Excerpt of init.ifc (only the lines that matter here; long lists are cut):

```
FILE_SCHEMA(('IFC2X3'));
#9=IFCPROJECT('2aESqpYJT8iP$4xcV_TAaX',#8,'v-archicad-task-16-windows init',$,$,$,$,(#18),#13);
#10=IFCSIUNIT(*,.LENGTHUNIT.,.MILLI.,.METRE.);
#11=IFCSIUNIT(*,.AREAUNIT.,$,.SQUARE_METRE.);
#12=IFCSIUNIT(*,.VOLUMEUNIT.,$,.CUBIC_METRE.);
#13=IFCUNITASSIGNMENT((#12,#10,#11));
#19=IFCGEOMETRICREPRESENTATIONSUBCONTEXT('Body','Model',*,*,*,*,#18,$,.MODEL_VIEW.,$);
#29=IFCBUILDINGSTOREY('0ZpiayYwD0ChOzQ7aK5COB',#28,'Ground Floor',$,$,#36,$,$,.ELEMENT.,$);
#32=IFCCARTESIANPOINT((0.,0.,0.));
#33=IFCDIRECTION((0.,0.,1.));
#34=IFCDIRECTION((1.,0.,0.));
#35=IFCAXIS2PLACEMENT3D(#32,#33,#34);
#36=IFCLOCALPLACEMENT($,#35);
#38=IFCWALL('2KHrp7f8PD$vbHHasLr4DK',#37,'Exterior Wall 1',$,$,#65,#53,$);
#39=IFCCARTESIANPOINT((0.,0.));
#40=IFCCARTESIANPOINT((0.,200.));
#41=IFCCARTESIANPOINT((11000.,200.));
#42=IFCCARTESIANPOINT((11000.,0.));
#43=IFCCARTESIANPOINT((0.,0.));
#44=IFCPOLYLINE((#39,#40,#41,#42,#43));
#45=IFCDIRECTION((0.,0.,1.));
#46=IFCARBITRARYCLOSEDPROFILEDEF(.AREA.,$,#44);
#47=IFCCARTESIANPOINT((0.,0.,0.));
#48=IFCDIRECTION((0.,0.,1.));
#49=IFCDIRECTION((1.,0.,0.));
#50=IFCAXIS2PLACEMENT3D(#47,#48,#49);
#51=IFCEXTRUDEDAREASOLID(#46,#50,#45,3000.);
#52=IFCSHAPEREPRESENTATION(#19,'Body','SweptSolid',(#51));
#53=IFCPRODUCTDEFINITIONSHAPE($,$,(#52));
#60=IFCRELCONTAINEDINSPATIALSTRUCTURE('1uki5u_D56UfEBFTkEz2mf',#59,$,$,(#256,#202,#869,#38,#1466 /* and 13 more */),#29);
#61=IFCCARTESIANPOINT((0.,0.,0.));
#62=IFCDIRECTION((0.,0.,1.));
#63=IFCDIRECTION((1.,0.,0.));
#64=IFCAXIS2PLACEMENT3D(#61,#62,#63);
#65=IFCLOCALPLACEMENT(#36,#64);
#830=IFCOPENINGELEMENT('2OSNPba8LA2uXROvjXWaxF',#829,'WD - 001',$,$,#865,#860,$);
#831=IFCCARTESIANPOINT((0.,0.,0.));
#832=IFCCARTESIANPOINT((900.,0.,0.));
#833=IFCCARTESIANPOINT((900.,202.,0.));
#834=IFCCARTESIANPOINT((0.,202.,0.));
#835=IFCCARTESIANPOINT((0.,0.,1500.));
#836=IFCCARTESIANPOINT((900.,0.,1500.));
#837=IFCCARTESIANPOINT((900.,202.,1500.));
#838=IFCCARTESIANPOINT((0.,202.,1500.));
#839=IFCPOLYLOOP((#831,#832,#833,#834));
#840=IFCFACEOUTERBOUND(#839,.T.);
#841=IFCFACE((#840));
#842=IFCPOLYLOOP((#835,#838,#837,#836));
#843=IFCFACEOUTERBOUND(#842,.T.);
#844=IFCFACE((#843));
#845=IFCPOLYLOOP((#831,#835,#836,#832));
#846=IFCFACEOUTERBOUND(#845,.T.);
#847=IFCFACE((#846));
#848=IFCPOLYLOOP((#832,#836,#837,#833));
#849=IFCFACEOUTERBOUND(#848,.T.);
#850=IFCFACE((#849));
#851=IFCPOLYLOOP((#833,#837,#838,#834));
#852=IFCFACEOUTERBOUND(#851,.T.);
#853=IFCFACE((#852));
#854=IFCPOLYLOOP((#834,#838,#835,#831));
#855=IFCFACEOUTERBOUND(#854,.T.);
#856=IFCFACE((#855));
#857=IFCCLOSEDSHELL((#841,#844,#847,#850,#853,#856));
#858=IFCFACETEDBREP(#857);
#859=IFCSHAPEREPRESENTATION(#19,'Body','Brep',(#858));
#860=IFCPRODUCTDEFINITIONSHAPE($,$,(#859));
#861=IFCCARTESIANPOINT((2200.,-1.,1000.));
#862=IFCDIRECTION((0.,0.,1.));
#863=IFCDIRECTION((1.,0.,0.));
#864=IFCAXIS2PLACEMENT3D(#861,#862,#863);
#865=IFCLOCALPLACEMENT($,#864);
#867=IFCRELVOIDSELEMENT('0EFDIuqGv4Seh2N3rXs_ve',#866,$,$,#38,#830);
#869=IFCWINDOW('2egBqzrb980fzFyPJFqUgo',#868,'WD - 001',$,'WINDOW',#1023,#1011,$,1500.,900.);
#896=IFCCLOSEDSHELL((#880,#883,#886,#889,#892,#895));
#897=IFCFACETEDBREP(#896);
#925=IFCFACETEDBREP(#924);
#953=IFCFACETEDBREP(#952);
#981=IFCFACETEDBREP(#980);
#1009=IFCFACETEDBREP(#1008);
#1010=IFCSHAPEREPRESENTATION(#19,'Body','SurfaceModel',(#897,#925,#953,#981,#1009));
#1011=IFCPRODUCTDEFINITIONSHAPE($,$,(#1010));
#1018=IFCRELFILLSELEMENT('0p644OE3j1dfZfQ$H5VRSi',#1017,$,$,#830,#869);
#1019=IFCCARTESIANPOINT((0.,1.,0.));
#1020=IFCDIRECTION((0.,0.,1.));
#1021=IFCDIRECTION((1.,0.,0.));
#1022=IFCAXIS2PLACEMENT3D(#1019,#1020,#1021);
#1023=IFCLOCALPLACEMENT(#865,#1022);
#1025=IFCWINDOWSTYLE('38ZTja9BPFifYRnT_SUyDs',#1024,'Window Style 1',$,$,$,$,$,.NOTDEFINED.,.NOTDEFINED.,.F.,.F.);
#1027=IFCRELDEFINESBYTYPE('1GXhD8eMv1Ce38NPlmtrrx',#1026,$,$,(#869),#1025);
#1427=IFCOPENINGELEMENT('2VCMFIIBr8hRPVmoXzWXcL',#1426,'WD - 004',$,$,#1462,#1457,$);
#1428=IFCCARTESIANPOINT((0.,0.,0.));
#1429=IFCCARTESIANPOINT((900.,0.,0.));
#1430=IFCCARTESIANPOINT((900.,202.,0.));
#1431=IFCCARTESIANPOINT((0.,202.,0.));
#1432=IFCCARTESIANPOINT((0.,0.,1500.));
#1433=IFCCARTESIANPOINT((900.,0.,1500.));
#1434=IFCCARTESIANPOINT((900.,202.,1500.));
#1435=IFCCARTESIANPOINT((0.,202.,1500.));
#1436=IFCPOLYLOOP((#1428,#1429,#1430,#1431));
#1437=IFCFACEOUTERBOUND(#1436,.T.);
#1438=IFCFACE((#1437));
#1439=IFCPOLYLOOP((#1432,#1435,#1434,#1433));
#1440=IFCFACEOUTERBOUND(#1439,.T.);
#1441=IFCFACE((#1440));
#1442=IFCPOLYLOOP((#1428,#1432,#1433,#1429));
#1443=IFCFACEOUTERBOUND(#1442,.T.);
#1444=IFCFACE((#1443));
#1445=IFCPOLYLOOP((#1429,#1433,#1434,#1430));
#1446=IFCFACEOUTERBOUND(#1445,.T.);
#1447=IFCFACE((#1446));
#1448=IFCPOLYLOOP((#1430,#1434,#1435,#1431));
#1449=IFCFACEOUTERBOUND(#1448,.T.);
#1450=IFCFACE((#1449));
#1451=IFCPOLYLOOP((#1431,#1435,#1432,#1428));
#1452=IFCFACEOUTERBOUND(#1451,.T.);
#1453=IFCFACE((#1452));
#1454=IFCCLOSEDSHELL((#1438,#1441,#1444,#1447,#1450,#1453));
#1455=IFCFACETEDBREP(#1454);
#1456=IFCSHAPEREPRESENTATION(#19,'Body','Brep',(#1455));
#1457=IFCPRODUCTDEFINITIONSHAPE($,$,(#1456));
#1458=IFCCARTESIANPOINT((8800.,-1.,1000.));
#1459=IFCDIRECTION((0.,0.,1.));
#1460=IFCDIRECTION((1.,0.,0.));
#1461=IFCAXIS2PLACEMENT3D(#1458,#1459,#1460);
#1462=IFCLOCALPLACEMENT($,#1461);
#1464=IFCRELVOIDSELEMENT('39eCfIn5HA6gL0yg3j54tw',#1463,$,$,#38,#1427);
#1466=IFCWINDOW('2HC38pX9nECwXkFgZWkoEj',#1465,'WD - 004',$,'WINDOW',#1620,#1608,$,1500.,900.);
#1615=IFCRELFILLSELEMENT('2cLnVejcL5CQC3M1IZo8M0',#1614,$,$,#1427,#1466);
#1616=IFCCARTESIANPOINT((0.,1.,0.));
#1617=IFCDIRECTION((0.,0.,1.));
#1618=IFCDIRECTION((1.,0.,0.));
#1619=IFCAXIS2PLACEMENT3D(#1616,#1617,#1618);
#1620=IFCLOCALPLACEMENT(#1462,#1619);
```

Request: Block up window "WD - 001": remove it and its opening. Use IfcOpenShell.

```python
import ifcopenshell
import ifcopenshell.api.feature
import ifcopenshell.api.root
import ifcopenshell.geom
import ifcopenshell.util.shape

model = ifcopenshell.open("init.ifc")
settings = ifcopenshell.geom.settings()


def volume(element):
    """Net volume in cubic metres, openings subtracted."""
    shape = ifcopenshell.geom.create_shape(settings, element)
    return ifcopenshell.util.shape.get_volume(shape.geometry)


window = model.by_guid("2egBqzrb980fzFyPJFqUgo")
opening = window.FillsVoids[0].RelatingOpeningElement
wall = opening.VoidsElements[0].RelatingBuildingElement
before = volume(wall)

ifcopenshell.api.root.remove_product(model, product=window)
ifcopenshell.api.feature.remove_feature(model, feature=opening)

after = volume(wall)

print(f"wall volume {before:.3f} -> {after:.3f} m3")

model.write("init_edited.ifc")
```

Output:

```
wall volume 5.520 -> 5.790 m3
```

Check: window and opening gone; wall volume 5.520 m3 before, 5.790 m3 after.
